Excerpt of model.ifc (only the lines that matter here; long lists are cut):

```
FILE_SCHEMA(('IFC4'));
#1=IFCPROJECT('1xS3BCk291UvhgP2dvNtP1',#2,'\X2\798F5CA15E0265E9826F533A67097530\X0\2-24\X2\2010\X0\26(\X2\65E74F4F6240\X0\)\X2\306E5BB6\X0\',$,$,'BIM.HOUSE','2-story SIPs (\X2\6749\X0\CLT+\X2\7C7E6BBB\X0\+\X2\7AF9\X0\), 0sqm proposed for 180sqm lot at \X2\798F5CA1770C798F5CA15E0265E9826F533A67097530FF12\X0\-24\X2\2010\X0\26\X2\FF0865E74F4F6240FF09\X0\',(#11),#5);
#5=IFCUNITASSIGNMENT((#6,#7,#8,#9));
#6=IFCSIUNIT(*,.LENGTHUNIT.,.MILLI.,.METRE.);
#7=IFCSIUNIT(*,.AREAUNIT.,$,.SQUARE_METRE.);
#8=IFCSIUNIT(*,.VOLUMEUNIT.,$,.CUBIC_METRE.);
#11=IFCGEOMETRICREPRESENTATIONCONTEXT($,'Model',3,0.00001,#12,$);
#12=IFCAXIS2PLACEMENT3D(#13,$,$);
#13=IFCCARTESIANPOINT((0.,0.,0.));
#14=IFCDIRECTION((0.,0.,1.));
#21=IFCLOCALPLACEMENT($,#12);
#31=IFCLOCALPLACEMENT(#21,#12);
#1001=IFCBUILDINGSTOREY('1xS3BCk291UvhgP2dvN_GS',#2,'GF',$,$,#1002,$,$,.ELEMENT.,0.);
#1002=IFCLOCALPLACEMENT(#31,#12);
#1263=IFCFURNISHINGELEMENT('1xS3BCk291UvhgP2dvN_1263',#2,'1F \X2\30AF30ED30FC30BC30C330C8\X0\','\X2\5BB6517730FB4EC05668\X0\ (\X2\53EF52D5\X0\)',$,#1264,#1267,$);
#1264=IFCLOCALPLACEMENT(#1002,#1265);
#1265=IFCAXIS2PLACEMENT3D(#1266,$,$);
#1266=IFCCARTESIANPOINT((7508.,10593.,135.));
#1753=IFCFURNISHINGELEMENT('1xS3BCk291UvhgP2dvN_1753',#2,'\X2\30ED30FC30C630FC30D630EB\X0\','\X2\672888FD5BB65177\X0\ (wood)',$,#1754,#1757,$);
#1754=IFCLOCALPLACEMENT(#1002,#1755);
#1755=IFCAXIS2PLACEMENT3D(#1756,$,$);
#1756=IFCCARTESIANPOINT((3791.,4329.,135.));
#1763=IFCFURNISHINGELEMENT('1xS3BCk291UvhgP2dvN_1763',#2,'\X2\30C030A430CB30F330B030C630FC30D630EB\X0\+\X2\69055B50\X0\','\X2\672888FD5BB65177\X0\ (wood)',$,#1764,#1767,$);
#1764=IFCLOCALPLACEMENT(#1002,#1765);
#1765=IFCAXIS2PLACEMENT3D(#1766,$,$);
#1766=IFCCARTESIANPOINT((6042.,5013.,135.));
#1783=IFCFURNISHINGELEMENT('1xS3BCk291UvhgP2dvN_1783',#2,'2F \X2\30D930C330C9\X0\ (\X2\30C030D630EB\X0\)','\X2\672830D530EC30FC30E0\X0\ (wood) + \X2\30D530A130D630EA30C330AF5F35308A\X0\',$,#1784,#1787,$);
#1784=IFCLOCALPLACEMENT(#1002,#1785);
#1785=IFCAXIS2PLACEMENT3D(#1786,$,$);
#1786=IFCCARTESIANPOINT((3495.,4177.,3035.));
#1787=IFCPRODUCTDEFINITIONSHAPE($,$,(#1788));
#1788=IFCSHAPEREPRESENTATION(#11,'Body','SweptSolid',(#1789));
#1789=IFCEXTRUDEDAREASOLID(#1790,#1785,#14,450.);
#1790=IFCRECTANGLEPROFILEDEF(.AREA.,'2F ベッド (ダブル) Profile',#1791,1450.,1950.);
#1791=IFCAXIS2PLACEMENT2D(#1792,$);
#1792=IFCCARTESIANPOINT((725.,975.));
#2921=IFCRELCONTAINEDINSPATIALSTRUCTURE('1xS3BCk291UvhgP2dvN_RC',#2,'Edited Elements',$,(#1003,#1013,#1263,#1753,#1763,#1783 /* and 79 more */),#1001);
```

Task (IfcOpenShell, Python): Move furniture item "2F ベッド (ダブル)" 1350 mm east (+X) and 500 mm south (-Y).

```python
import ifcopenshell
import ifcopenshell.api.geometry
import ifcopenshell.util.placement
import ifcopenshell.util.unit

model = ifcopenshell.open("model.ifc")
unit_scale = ifcopenshell.util.unit.calculate_unit_scale(model)

item = model.by_id(1783)
matrix = ifcopenshell.util.placement.get_local_placement(item.ObjectPlacement)
matrix[0, 3] += 1.35 / unit_scale
matrix[1, 3] -= 0.5 / unit_scale
ifcopenshell.api.geometry.edit_object_placement(model, product=item, matrix=matrix, is_si=False)

print(ifcopenshell.util.placement.get_local_placement(item.ObjectPlacement).round(3) + 0.0)

model.write("model-out.ifc")
```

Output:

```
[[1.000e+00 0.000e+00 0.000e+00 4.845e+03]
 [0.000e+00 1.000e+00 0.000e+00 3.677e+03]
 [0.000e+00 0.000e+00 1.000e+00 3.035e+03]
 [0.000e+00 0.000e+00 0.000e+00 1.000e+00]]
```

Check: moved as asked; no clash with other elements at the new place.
